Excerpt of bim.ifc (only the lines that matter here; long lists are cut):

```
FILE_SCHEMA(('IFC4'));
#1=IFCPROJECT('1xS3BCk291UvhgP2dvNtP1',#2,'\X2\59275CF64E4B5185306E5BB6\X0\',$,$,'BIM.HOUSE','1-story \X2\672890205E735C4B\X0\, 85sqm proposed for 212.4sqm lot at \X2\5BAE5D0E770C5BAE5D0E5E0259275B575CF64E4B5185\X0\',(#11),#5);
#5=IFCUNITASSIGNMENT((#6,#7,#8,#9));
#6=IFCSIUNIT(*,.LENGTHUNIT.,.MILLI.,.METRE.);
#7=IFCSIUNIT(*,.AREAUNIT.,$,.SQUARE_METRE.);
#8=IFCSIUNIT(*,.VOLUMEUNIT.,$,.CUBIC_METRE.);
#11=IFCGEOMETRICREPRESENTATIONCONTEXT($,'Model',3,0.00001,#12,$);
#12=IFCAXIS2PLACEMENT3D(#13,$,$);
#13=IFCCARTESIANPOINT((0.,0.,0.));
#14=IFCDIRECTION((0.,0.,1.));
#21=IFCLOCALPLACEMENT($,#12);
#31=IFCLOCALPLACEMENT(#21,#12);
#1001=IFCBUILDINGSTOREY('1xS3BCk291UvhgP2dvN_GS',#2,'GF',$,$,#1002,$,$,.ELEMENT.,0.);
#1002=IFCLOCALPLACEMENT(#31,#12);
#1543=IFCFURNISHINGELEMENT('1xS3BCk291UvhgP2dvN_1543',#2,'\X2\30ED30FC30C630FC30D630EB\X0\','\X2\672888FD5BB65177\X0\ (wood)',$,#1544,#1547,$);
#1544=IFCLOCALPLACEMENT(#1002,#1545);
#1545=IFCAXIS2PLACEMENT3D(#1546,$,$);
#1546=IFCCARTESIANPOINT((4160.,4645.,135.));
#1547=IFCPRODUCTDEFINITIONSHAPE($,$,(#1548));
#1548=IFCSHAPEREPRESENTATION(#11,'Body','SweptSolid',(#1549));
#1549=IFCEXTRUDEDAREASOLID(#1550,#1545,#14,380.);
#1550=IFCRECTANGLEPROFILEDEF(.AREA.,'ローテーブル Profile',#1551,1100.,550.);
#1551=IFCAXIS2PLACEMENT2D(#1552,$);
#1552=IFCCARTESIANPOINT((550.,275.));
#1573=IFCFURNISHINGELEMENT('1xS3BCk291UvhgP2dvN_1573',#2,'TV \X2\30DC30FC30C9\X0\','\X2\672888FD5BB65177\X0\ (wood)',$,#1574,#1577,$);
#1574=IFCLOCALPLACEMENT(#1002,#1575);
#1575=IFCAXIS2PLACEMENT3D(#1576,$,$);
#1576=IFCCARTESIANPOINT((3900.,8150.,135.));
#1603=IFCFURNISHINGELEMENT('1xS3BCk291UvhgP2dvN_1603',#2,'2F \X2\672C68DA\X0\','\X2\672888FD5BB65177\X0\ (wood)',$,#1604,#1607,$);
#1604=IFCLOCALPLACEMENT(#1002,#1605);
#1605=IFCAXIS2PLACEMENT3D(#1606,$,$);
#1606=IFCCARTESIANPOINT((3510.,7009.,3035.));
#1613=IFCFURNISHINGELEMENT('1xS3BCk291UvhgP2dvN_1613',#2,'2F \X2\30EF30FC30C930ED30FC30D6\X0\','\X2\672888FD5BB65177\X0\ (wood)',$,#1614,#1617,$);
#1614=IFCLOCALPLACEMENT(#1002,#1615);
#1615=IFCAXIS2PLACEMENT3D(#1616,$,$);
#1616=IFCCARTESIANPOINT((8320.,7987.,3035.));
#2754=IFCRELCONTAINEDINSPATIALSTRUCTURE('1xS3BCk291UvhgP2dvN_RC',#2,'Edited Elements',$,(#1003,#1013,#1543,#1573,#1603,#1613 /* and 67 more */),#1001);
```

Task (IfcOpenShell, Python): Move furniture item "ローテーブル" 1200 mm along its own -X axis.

```python
import ifcopenshell
import ifcopenshell.api.geometry
import ifcopenshell.util.placement
import ifcopenshell.util.unit

model = ifcopenshell.open("bim.ifc")
unit_scale = ifcopenshell.util.unit.calculate_unit_scale(model)

item = model.by_guid("1xS3BCk291UvhgP2dvN_1543")
matrix = ifcopenshell.util.placement.get_local_placement(item.ObjectPlacement)
matrix[:3, 3] -= matrix[:3, 0] * 1.2 / unit_scale
ifcopenshell.api.geometry.edit_object_placement(model, product=item, matrix=matrix, is_si=False)

print(ifcopenshell.util.placement.get_local_placement(item.ObjectPlacement).round(3) + 0.0)

model.write("bim_edited.ifc")
```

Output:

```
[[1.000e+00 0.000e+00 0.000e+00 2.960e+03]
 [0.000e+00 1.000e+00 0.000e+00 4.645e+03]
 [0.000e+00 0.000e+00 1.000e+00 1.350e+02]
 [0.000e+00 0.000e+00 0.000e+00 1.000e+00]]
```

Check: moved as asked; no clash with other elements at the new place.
